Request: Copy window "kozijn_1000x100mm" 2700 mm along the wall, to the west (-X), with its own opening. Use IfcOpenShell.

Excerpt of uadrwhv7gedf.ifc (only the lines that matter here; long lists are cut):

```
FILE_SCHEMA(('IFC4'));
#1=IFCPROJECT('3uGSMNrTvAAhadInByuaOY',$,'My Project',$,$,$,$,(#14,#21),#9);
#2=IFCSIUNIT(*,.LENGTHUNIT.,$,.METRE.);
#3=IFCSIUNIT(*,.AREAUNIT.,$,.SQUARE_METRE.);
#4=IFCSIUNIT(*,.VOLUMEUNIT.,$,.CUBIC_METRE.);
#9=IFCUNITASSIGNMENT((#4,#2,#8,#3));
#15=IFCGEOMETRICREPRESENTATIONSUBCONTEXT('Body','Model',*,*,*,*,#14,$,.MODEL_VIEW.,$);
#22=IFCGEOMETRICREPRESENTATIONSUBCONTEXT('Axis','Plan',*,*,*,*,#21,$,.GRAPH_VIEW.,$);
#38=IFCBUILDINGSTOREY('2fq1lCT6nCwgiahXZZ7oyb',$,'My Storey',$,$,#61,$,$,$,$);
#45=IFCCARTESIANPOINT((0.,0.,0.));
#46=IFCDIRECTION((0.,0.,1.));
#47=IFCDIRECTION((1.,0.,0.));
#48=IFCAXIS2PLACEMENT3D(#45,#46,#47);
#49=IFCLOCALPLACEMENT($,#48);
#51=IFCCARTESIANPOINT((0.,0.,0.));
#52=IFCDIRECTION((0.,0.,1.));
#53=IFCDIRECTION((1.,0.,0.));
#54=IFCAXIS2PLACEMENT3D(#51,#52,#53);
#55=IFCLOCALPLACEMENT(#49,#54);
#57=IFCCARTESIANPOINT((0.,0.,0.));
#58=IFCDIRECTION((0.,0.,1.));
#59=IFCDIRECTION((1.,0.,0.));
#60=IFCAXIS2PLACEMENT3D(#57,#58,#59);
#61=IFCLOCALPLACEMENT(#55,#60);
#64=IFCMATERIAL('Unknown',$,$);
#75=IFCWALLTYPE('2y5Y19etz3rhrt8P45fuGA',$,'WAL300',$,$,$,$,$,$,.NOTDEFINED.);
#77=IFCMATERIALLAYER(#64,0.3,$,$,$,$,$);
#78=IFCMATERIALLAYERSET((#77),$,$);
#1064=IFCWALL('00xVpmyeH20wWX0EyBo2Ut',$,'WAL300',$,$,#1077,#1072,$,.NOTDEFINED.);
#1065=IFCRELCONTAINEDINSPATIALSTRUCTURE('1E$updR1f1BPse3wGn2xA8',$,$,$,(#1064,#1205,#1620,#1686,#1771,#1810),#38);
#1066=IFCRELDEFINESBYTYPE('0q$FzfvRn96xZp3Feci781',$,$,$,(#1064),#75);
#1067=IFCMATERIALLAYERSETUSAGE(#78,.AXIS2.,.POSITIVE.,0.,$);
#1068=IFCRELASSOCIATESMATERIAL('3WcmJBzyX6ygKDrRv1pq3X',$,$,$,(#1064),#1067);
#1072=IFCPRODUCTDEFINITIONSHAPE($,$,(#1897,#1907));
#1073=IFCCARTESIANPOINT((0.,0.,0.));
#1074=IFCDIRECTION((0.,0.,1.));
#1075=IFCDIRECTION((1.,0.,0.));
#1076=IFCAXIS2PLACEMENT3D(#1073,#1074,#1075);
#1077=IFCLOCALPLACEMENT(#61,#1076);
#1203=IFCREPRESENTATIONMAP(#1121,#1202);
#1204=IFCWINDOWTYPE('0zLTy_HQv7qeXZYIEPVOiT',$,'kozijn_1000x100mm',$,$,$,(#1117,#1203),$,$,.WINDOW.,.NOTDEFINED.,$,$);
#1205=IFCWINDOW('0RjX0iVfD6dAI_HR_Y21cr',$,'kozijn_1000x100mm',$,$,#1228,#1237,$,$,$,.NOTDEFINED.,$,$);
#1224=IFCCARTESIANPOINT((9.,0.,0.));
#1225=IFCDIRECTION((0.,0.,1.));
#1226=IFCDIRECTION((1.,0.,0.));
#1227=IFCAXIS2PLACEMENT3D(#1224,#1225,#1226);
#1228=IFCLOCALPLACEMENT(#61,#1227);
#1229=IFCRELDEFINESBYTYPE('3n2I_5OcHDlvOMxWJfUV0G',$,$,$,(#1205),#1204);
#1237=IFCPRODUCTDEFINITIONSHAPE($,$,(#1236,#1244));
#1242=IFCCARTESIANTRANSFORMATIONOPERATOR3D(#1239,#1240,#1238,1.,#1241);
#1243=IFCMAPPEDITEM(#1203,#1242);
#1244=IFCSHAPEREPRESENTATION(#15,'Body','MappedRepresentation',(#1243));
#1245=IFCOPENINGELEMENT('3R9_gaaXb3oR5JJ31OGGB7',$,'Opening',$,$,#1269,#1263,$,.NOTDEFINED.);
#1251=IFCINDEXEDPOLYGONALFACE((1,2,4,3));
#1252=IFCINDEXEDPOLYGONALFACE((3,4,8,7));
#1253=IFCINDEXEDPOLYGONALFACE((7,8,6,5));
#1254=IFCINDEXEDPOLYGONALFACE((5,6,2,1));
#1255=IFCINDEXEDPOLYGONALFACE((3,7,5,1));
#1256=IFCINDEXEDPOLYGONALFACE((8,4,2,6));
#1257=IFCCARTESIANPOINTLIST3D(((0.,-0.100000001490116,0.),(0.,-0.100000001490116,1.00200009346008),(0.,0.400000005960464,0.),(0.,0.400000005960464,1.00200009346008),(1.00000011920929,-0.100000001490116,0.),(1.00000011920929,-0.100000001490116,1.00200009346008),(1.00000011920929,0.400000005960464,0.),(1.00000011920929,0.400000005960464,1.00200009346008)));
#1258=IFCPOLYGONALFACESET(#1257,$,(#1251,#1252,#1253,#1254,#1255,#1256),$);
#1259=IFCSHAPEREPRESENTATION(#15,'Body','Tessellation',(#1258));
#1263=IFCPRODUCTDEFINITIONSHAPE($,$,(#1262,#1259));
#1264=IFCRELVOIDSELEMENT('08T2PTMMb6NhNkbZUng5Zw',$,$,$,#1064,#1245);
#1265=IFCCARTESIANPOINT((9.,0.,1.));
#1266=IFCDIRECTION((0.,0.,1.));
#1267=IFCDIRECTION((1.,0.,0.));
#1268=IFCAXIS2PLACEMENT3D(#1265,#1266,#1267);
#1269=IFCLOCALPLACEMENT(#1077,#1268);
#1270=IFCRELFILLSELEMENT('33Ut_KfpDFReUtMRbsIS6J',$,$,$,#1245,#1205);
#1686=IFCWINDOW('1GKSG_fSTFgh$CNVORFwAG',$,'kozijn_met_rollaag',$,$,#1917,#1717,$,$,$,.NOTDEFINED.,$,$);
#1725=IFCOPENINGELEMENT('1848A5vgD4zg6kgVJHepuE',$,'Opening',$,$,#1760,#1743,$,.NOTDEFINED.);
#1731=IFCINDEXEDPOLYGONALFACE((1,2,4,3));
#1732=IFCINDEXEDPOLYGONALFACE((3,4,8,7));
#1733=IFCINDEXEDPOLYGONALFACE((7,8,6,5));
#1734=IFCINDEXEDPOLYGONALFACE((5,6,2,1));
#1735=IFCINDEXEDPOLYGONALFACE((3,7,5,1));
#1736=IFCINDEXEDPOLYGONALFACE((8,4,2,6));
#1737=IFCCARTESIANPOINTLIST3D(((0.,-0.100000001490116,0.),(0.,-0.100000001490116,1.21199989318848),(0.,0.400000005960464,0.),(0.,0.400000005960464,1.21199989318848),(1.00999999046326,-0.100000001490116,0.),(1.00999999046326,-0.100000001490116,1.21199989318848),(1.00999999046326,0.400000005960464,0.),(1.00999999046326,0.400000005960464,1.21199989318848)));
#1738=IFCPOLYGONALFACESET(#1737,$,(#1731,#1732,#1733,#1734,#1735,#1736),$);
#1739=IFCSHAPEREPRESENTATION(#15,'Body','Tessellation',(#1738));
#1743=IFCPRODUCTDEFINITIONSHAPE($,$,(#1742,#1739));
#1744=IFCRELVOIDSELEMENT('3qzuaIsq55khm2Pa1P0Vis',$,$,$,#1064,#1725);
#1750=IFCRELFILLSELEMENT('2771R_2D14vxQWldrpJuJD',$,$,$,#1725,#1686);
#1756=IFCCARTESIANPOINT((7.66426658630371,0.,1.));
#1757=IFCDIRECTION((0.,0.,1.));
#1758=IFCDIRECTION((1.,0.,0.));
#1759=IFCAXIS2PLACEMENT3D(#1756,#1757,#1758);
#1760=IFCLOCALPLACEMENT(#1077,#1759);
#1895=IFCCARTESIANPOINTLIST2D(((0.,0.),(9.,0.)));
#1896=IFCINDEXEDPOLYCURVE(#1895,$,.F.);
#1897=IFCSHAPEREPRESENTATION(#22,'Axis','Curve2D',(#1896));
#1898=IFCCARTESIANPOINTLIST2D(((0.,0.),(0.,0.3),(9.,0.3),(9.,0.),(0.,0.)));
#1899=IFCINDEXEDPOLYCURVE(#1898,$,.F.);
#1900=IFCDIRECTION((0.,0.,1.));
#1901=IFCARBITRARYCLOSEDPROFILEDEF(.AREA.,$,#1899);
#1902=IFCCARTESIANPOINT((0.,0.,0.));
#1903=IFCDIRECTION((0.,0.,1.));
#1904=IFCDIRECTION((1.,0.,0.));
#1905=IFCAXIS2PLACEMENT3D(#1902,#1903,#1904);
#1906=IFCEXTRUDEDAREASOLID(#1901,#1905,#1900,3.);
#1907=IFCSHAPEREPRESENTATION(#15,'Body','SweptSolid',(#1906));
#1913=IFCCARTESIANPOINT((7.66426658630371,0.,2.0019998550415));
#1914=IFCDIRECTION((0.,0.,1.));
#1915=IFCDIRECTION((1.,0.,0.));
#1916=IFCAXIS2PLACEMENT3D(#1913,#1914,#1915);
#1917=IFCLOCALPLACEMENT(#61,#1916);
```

```python
import ifcopenshell
import ifcopenshell.api.feature
import ifcopenshell.api.geometry
import ifcopenshell.api.root
import ifcopenshell.geom
import ifcopenshell.util.element
import ifcopenshell.util.placement
import ifcopenshell.util.shape
import ifcopenshell.util.unit

model = ifcopenshell.open("uadrwhv7gedf.ifc")
unit_scale = ifcopenshell.util.unit.calculate_unit_scale(model)
settings = ifcopenshell.geom.settings()


def volume(element):
    """Net volume in cubic metres, openings subtracted."""
    shape = ifcopenshell.geom.create_shape(settings, element)
    return ifcopenshell.util.shape.get_volume(shape.geometry)


window = model.by_id(1205)
opening = window.FillsVoids[0].RelatingOpeningElement
wall = opening.VoidsElements[0].RelatingBuildingElement
before = volume(wall)
shift = ifcopenshell.util.placement.get_local_placement(wall.ObjectPlacement)[:3, 0] * -2.7 / unit_scale

# copy_class copies the void relationship, type, container and properties, but no geometry.
new_opening = ifcopenshell.api.root.copy_class(model, product=opening)
new_opening.Representation = ifcopenshell.util.element.copy_deep(
    model, opening.Representation, exclude=["IfcGeometricRepresentationContext", "IfcRepresentationMap"]
)
new_window = ifcopenshell.api.root.copy_class(model, product=window)
new_window.Representation = ifcopenshell.util.element.copy_deep(
    model, window.Representation, exclude=["IfcGeometricRepresentationContext", "IfcRepresentationMap"]
)
ifcopenshell.api.feature.add_filling(model, opening=new_opening, element=new_window)

for old, new in ((opening, new_opening), (window, new_window)):
    matrix = ifcopenshell.util.placement.get_local_placement(old.ObjectPlacement)
    matrix[:3, 3] += shift
    ifcopenshell.api.geometry.edit_object_placement(model, product=new, matrix=matrix, is_si=False)

after = volume(wall)

print(f"wall volume {before:.3f} -> {after:.3f} m3")

model.write("uadrwhv7gedf-out.ifc")
```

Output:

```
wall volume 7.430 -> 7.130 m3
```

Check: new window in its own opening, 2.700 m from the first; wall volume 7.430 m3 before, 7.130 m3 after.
